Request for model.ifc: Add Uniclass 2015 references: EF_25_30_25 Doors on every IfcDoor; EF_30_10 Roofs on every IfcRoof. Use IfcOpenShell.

First a look at what the model holds.

```python
import ifcopenshell

model = ifcopenshell.open("model.ifc")
print(model.schema)
print("classifications:", [c.Name for c in model.by_type("IfcClassification")])
for ifc_class in ("IfcDoor", "IfcRoof", "IfcStair", "IfcWall", "IfcWindow"):
    print(ifc_class, len(model.by_type(ifc_class)))
```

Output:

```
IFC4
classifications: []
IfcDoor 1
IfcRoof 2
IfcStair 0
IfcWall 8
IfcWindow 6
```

```python
import ifcopenshell
import ifcopenshell.api.classification

model = ifcopenshell.open("model.ifc")

system = ifcopenshell.api.classification.add_classification(model, classification="Uniclass 2015")

codes = {
    "IfcDoor": ("EF_25_30_25", "Doors"),
    "IfcRoof": ("EF_30_10", "Roofs"),
}
for ifc_class, (code, name) in codes.items():
    products = model.by_type(ifc_class)
    ifcopenshell.api.classification.add_reference(
        model, products=products, classification=system, identification=code, name=name
    )
    print(code, len(products))

model.write("model_v2.ifc")
```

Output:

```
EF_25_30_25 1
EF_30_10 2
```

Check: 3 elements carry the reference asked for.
